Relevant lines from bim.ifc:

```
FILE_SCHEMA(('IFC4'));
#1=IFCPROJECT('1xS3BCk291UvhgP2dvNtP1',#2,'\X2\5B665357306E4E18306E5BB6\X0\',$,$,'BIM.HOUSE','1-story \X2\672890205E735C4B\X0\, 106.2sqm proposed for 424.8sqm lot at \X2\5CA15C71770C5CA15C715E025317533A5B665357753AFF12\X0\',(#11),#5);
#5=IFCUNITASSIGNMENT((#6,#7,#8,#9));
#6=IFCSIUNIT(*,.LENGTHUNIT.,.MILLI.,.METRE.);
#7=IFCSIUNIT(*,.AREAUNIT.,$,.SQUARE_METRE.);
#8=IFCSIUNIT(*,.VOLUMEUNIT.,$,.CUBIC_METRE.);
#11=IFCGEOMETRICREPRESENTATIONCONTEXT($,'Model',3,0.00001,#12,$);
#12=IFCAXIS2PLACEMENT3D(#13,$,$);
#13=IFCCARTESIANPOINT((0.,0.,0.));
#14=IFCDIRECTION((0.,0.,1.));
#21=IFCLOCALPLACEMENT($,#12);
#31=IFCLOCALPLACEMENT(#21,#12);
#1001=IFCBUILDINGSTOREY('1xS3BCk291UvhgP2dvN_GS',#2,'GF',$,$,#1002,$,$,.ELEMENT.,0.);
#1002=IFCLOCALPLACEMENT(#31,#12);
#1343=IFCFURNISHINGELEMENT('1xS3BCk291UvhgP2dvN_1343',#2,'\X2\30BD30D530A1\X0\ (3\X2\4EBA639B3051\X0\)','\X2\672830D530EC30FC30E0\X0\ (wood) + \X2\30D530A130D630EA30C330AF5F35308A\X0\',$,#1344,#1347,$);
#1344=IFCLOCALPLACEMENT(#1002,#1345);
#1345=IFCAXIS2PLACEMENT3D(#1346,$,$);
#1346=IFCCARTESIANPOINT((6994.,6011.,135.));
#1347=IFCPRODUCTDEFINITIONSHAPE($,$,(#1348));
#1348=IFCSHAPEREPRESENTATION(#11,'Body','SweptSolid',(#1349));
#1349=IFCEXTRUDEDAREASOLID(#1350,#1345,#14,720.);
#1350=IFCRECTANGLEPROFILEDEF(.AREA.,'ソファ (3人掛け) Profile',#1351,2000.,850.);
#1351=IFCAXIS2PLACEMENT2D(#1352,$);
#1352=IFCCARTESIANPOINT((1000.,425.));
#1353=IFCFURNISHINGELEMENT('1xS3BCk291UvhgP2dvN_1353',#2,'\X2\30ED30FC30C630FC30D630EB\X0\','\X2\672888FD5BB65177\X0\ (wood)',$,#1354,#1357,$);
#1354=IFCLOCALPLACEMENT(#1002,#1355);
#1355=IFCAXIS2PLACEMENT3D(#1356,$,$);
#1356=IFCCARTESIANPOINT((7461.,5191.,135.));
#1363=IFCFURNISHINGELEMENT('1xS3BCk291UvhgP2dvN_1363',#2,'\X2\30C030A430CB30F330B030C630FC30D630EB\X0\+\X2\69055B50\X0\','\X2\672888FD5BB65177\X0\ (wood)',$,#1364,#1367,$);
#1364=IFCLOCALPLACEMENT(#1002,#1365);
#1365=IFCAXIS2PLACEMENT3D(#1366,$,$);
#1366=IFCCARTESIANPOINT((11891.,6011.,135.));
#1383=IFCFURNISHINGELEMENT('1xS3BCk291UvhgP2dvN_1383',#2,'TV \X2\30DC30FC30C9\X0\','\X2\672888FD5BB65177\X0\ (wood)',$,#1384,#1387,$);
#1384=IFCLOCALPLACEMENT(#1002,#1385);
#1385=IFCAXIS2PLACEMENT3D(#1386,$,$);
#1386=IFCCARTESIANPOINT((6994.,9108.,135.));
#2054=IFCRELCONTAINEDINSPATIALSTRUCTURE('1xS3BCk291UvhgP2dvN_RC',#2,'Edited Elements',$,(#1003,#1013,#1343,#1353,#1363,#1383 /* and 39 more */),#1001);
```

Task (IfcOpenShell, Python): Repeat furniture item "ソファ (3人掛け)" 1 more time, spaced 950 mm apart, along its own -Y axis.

```python
import ifcopenshell
import ifcopenshell.api.geometry
import ifcopenshell.api.root
import ifcopenshell.util.element
import ifcopenshell.util.placement

model = ifcopenshell.open("bim.ifc")


def reuse_history(source, copy):
    """copy_class also copies each property set's owner history, people and application; keep the originals."""
    for rel in copy.IsDefinedBy:
        if rel.is_a("IfcRelDefinesByProperties") and (history := rel.RelatingPropertyDefinition.OwnerHistory):
            rel.RelatingPropertyDefinition.OwnerHistory = source.OwnerHistory
            ifcopenshell.util.element.remove_deep2(model, history)


source = model.by_id(1343)
base = ifcopenshell.util.placement.get_local_placement(source.ObjectPlacement)
step = -base[:3, 1] * 950.0

for i in range(1, 2):
    copy = ifcopenshell.api.root.copy_class(model, product=source)
    copy.Representation = ifcopenshell.util.element.copy_deep(
        model, source.Representation, exclude=["IfcGeometricRepresentationContext", "IfcRepresentationMap"]
    )
    reuse_history(source, copy)
    matrix = base.copy()
    matrix[:3, 3] += i * step
    print("added at", matrix[:3, 3].round(3) + 0.0)
    ifcopenshell.api.geometry.edit_object_placement(model, product=copy, matrix=matrix, is_si=False)

model.write("bim_edited.ifc")
```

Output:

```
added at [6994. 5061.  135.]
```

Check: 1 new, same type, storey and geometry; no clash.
